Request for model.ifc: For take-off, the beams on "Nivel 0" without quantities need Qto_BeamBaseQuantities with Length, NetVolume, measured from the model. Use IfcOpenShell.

First a look at what the model holds.

```python
import ifcopenshell
import ifcopenshell.util.element
import ifcopenshell.util.unit

model = ifcopenshell.open("model.ifc")
print(model.schema)
for unit_type in ("LENGTHUNIT", "AREAUNIT", "VOLUMEUNIT"):
    print(unit_type, ifcopenshell.util.unit.calculate_unit_scale(model, unit_type))
storey = next(s for s in model.by_type("IfcBuildingStorey") if s.Name == "Nivel 0")
beams = [e for e in ifcopenshell.util.element.get_decomposition(storey) if e.is_a("IfcBeam")]
for e in sorted(beams, key=lambda e: e.id()):
    print(e.id(), e.is_a(), e.Name, list(ifcopenshell.util.element.get_psets(e, qtos_only=True)), sep=" | ")
```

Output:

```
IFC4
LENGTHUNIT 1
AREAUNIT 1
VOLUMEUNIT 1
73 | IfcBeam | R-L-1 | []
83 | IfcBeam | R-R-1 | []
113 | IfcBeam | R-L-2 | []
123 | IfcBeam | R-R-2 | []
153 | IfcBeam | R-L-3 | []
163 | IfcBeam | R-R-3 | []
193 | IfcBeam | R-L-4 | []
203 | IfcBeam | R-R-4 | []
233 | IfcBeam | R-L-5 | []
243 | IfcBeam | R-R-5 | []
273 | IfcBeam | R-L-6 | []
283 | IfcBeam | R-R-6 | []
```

```python
import ifcopenshell
import ifcopenshell.api.pset
import ifcopenshell.geom
import ifcopenshell.util.element
import ifcopenshell.util.shape
import ifcopenshell.util.unit

model = ifcopenshell.open("model.ifc")
unit_scale = ifcopenshell.util.unit.calculate_unit_scale(model)
volume_scale = ifcopenshell.util.unit.calculate_unit_scale(model, "VOLUMEUNIT")
settings = ifcopenshell.geom.settings()

storey = next(s for s in model.by_type("IfcBuildingStorey") if s.Name == "Nivel 0")
beams = [e for e in ifcopenshell.util.element.get_decomposition(storey) if e.is_a("IfcBeam")]

for e in sorted(beams, key=lambda e: e.id()):
    if ifcopenshell.util.element.get_psets(e, qtos_only=True, should_inherit=False):
        continue
    # Geometry comes back in metres, in the element's own axes.
    shape = ifcopenshell.geom.create_shape(settings, e)
    values = {
        "Length": ifcopenshell.util.shape.get_max_xyz(shape.geometry) / unit_scale,
        "NetVolume": ifcopenshell.util.shape.get_volume(shape.geometry) / volume_scale,
    }
    qto = ifcopenshell.api.pset.add_qto(model, product=e, name="Qto_BeamBaseQuantities")
    ifcopenshell.api.pset.edit_qto(model, qto=qto, properties=values)
    print(e.id(), {k: round(v, 3) for k, v in values.items()})

model.write("model_updated.ifc")
```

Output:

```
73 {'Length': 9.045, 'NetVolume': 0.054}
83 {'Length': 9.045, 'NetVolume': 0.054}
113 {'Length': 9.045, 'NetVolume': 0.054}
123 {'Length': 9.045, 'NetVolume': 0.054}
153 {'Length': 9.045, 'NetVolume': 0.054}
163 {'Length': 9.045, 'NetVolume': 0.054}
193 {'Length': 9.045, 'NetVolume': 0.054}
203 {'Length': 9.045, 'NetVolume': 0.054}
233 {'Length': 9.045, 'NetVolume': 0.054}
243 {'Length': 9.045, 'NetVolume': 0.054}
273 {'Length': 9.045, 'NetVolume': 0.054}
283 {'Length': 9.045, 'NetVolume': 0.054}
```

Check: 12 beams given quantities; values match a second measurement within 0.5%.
